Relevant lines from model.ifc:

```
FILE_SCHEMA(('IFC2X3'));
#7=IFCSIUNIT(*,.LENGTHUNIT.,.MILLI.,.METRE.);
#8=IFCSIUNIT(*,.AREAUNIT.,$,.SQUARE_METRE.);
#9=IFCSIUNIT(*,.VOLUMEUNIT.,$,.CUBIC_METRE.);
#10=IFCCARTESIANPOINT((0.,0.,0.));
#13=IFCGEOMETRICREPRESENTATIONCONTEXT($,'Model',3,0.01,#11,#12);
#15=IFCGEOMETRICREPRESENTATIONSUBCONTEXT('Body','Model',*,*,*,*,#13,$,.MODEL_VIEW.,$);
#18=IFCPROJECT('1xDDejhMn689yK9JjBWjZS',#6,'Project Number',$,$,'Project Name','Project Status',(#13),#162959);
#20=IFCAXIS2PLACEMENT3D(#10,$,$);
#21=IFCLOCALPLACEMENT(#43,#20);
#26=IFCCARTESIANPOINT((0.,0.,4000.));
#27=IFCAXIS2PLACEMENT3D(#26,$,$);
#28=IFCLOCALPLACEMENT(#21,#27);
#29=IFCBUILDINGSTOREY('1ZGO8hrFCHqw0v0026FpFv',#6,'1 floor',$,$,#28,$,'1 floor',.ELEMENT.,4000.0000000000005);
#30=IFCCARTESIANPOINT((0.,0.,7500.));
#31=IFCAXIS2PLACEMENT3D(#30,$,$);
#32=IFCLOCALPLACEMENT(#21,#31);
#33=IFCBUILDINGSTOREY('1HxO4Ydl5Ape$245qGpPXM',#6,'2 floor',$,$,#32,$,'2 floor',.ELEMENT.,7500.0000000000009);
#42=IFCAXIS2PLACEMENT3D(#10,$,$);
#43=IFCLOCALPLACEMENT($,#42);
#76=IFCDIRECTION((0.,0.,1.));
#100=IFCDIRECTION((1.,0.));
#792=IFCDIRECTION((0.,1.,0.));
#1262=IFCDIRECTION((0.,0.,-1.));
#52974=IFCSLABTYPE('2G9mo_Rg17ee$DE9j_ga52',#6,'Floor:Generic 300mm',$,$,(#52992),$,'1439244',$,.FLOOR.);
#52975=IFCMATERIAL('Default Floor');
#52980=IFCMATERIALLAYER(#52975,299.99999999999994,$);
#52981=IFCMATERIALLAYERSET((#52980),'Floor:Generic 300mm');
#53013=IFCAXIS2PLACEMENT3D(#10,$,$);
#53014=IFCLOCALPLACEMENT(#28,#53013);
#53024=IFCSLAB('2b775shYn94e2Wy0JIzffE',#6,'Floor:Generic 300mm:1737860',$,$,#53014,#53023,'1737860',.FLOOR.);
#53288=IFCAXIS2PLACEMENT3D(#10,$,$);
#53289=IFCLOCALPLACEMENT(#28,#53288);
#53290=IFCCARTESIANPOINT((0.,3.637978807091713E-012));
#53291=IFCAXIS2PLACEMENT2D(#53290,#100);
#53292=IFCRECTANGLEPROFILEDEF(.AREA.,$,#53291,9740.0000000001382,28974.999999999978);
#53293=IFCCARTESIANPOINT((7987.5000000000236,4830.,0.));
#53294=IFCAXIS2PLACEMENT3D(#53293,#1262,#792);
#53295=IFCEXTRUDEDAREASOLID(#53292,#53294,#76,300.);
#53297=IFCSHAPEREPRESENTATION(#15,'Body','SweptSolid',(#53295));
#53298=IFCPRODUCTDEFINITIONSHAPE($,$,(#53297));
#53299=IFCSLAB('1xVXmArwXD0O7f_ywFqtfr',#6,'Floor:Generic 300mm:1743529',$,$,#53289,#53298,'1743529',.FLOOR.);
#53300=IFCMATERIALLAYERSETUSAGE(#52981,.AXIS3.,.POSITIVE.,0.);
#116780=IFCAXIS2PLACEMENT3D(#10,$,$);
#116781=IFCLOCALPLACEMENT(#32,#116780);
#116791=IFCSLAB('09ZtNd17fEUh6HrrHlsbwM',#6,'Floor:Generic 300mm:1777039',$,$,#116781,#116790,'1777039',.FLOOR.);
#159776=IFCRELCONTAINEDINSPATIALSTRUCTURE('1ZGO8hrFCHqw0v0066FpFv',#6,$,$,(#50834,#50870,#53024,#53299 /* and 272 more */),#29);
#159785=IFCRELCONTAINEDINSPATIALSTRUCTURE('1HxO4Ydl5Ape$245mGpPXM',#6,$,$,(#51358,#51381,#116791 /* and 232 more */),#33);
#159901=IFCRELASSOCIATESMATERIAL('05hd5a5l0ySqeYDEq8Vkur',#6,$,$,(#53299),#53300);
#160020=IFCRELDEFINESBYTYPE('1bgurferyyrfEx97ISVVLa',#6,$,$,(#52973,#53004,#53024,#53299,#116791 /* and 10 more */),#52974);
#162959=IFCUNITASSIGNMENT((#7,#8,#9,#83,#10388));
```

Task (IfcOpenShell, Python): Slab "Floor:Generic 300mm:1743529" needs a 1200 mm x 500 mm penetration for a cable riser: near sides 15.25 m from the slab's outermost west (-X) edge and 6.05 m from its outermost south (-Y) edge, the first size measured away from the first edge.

```python
import numpy as np
import ifcopenshell
import ifcopenshell.api.feature
import ifcopenshell.api.geometry
import ifcopenshell.api.root
import ifcopenshell.geom
import ifcopenshell.util.placement
import ifcopenshell.util.representation
import ifcopenshell.util.shape
import ifcopenshell.util.unit

model = ifcopenshell.open("model.ifc")
unit_scale = ifcopenshell.util.unit.calculate_unit_scale(model)
settings = ifcopenshell.geom.settings()


def volume(element):
    """Net volume in cubic metres, openings subtracted."""
    shape = ifcopenshell.geom.create_shape(settings, element)
    return ifcopenshell.util.shape.get_volume(shape.geometry)


slab = model.by_id(53299)
before = volume(slab)

# Extent in the slab's own axes, in metres. The edges named are its -X and -Y sides.
slab_shape = ifcopenshell.geom.create_shape(settings, slab)
vertices = ifcopenshell.util.shape.get_vertices(slab_shape.geometry)
x_min, y_min, bottom = vertices.min(axis=0)
top = vertices[:, 2].max()

opening = ifcopenshell.api.root.create_entity(model, ifc_class="IfcOpeningElement", name="Cable riser opening")
context = ifcopenshell.util.representation.get_context(model, "Model", "Body", "MODEL_VIEW")
width, depth = 1.2, 0.5
outline = [(0.0, 0.0), (width, 0.0), (width, depth), (0.0, depth), (0.0, 0.0)]
# Overshoot both faces by 50 mm so the cut is clean.
shape = ifcopenshell.api.geometry.add_slab_representation(
    model, context=context, depth=top - bottom + 0.1, polyline=outline
)
ifcopenshell.api.geometry.assign_representation(model, product=opening, representation=shape)

matrix = ifcopenshell.util.placement.get_local_placement(slab.ObjectPlacement)
matrix[:, 3] = matrix @ np.append(np.array([x_min + 15.25, y_min + 6.05, bottom - 0.05]) / unit_scale, 1.0)
ifcopenshell.api.geometry.edit_object_placement(model, product=opening, matrix=matrix, is_si=False)
ifcopenshell.api.feature.add_feature(model, feature=opening, element=slab)

after = volume(slab)

print(f"slab volume {before:.3f} -> {after:.3f} m3")

model.write("model_rev.ifc")
```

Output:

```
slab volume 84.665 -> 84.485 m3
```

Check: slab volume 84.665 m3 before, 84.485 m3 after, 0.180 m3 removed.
